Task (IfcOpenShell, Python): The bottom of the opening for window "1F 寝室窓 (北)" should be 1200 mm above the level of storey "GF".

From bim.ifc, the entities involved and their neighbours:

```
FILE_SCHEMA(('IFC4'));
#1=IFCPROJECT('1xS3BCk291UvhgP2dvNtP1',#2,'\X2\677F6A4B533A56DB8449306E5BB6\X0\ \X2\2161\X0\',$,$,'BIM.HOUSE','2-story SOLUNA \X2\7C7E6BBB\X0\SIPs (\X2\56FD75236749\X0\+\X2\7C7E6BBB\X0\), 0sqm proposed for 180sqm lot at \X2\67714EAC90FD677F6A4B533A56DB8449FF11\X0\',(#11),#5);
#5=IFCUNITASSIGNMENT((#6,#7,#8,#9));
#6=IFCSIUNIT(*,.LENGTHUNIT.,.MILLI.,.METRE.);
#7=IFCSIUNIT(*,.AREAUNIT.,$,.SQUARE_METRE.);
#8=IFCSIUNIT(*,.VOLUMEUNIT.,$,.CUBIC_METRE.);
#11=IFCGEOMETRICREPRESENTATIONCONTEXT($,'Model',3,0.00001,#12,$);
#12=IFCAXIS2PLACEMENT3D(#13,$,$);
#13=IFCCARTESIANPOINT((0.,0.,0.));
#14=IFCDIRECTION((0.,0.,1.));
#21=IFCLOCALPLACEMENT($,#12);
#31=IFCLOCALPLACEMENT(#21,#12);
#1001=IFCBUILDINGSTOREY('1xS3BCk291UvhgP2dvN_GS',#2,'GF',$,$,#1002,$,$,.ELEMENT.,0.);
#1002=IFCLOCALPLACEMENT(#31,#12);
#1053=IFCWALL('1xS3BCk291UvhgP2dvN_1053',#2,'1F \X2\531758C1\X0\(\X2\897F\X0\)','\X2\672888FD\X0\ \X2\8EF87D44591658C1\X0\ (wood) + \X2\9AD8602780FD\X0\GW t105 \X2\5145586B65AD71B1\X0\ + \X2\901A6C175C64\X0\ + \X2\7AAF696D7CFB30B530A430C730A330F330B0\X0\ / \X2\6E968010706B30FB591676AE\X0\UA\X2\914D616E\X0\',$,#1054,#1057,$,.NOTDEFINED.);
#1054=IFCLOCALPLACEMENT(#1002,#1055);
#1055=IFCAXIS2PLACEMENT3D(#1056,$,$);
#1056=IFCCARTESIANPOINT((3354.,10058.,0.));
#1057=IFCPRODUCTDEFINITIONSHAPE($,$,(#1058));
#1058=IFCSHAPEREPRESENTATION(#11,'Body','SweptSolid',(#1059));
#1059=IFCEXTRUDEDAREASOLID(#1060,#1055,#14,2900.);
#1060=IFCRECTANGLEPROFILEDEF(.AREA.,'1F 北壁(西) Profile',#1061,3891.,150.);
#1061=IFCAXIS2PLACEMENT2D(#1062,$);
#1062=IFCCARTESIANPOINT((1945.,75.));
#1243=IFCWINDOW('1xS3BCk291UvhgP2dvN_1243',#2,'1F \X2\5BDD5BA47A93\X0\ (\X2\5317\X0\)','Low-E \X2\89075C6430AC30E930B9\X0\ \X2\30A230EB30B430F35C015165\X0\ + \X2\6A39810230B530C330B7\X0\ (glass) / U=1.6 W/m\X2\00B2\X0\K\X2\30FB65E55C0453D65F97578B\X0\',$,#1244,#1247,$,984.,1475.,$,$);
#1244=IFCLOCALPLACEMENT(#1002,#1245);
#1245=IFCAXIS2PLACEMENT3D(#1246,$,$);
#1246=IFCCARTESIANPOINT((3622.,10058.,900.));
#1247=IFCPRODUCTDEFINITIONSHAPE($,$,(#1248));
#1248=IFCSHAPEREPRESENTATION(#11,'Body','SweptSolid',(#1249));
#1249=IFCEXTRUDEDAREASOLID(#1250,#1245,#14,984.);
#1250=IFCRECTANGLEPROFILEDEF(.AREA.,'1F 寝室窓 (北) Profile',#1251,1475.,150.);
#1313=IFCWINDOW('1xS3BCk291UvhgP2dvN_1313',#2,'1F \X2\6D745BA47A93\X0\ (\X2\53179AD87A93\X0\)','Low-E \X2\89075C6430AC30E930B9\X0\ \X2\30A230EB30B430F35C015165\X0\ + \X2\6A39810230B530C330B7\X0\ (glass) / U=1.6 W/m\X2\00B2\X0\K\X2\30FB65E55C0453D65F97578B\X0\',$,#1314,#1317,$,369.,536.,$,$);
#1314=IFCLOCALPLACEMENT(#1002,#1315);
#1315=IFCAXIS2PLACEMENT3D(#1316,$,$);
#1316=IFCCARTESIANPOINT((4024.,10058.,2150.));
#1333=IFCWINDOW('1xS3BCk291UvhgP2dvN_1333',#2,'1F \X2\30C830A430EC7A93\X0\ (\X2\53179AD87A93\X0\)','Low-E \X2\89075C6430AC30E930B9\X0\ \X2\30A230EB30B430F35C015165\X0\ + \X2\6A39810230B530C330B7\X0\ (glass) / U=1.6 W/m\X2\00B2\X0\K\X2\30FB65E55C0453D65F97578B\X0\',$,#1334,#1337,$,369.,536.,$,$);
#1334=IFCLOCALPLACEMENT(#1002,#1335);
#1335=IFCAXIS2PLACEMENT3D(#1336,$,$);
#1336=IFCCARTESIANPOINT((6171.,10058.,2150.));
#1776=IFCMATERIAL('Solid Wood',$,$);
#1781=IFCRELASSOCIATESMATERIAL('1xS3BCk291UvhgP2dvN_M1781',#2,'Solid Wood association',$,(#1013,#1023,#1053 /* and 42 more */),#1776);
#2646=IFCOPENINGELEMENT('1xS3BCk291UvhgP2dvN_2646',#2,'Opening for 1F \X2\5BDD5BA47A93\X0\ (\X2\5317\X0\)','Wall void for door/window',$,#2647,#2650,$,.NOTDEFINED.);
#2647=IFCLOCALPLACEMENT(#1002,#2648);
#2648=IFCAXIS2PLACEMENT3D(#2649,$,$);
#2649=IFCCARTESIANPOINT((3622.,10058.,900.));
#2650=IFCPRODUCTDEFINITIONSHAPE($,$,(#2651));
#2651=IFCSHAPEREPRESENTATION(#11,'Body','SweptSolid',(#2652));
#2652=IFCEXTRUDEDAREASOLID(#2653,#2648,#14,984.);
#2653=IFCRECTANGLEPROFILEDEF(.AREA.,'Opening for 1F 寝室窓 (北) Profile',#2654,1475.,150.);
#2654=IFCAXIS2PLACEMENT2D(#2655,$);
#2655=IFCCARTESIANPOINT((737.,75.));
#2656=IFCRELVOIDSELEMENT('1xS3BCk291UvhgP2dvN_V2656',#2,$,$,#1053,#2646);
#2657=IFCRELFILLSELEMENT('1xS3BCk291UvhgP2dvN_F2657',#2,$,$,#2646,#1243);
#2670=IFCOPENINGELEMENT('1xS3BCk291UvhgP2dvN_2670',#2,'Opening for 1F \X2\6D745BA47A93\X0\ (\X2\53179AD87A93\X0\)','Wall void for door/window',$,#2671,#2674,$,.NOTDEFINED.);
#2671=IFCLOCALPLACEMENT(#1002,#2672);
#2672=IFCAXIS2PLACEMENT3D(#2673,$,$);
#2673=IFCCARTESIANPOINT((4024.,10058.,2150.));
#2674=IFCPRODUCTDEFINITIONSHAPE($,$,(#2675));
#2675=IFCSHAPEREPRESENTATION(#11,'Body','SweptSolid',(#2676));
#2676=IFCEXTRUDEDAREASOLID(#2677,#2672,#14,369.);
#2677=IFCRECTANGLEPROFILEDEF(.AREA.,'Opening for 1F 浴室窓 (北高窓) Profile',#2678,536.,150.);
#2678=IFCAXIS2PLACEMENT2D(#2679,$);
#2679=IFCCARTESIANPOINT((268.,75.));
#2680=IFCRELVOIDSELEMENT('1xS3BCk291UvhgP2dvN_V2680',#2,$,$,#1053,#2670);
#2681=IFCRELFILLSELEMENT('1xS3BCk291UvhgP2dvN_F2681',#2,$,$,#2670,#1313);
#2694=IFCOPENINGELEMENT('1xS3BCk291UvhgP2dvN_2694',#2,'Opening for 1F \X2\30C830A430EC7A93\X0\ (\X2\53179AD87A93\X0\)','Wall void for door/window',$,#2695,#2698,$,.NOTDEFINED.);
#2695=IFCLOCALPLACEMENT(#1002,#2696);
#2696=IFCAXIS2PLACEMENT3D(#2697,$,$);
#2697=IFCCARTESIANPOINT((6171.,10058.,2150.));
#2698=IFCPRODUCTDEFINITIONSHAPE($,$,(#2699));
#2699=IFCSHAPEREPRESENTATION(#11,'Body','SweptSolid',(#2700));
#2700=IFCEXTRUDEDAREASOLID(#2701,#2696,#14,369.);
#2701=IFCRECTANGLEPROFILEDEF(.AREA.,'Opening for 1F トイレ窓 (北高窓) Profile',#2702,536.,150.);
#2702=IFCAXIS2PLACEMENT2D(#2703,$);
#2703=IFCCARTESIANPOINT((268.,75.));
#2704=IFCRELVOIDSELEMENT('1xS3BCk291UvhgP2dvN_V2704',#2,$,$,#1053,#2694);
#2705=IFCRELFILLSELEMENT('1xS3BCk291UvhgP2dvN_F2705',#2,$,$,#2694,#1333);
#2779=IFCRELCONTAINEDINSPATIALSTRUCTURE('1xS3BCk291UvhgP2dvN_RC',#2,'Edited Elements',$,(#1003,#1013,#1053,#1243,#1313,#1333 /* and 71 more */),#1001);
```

```python
import numpy as np
import ifcopenshell
import ifcopenshell.api.geometry
import ifcopenshell.geom
import ifcopenshell.util.element
import ifcopenshell.util.placement
import ifcopenshell.util.shape
import ifcopenshell.util.unit

model = ifcopenshell.open("bim.ifc")
unit_scale = ifcopenshell.util.unit.calculate_unit_scale(model)

window = model.by_guid("1xS3BCk291UvhgP2dvN_1243")
opening = window.FillsVoids[0].RelatingOpeningElement
storey = ifcopenshell.util.element.get_container(window, ifc_class="IfcBuildingStorey")
level = ifcopenshell.util.placement.get_local_placement(storey.ObjectPlacement)[2, 3]

# The opening's origin need not be at the sill, so measure its lowest point.
shape = ifcopenshell.geom.create_shape(ifcopenshell.geom.settings(), opening)
bottom = ifcopenshell.util.shape.get_shape_bottom_elevation(shape, shape.geometry) / unit_scale
dz = level + 1.2 / unit_scale - bottom

shift = np.array([0.0, 0.0, dz])
# The window is not placed relative to its opening, so move both.
for product in (opening, window):
    matrix = ifcopenshell.util.placement.get_local_placement(product.ObjectPlacement)
    matrix[:3, 3] += shift
    ifcopenshell.api.geometry.edit_object_placement(model, product=product, matrix=matrix, is_si=False)

print(f"moved by {dz * unit_scale:+.3f} m")

model.write("bim_rev.ifc")
```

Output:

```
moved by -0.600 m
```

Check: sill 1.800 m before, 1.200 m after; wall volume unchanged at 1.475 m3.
